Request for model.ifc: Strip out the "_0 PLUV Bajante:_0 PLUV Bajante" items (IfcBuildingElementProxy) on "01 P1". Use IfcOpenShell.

First a look at what the model holds.

```python
import ifcopenshell
import ifcopenshell.util.element

model = ifcopenshell.open("model.ifc")
print(model.schema)
storey = next(s for s in model.by_type("IfcBuildingStorey") if s.Name == "01 P1")
proxies = [e for e in ifcopenshell.util.element.get_decomposition(storey) if e.is_a("IfcBuildingElementProxy")]
seen = {}
for e in proxies:
    element_type = ifcopenshell.util.element.get_type(e)
    name = element_type.Name if element_type not in (None, e) else None
    seen[name] = seen.get(name, 0) + 1
for name, count in sorted(seen.items(), key=str):
    print(count, "x", name)
```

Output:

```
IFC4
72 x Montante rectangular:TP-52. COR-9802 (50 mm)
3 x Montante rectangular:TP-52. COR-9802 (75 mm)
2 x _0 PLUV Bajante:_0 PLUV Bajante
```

```python
import ifcopenshell
import ifcopenshell.api.root
import ifcopenshell.util.element

model = ifcopenshell.open("model.ifc")

storey = next(s for s in model.by_type("IfcBuildingStorey") if s.Name == "01 P1")
proxies = [e for e in ifcopenshell.util.element.get_decomposition(storey) if e.is_a("IfcBuildingElementProxy")]
targets = [e for e in proxies if (t := ifcopenshell.util.element.get_type(e)) not in (None, e) and t.Name == "_0 PLUV Bajante:_0 PLUV Bajante"]

for e in targets:
    ifcopenshell.api.root.remove_product(model, product=e)
print(len(targets), "removed")

model.write("model_rev.ifc")
```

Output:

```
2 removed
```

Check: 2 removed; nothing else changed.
